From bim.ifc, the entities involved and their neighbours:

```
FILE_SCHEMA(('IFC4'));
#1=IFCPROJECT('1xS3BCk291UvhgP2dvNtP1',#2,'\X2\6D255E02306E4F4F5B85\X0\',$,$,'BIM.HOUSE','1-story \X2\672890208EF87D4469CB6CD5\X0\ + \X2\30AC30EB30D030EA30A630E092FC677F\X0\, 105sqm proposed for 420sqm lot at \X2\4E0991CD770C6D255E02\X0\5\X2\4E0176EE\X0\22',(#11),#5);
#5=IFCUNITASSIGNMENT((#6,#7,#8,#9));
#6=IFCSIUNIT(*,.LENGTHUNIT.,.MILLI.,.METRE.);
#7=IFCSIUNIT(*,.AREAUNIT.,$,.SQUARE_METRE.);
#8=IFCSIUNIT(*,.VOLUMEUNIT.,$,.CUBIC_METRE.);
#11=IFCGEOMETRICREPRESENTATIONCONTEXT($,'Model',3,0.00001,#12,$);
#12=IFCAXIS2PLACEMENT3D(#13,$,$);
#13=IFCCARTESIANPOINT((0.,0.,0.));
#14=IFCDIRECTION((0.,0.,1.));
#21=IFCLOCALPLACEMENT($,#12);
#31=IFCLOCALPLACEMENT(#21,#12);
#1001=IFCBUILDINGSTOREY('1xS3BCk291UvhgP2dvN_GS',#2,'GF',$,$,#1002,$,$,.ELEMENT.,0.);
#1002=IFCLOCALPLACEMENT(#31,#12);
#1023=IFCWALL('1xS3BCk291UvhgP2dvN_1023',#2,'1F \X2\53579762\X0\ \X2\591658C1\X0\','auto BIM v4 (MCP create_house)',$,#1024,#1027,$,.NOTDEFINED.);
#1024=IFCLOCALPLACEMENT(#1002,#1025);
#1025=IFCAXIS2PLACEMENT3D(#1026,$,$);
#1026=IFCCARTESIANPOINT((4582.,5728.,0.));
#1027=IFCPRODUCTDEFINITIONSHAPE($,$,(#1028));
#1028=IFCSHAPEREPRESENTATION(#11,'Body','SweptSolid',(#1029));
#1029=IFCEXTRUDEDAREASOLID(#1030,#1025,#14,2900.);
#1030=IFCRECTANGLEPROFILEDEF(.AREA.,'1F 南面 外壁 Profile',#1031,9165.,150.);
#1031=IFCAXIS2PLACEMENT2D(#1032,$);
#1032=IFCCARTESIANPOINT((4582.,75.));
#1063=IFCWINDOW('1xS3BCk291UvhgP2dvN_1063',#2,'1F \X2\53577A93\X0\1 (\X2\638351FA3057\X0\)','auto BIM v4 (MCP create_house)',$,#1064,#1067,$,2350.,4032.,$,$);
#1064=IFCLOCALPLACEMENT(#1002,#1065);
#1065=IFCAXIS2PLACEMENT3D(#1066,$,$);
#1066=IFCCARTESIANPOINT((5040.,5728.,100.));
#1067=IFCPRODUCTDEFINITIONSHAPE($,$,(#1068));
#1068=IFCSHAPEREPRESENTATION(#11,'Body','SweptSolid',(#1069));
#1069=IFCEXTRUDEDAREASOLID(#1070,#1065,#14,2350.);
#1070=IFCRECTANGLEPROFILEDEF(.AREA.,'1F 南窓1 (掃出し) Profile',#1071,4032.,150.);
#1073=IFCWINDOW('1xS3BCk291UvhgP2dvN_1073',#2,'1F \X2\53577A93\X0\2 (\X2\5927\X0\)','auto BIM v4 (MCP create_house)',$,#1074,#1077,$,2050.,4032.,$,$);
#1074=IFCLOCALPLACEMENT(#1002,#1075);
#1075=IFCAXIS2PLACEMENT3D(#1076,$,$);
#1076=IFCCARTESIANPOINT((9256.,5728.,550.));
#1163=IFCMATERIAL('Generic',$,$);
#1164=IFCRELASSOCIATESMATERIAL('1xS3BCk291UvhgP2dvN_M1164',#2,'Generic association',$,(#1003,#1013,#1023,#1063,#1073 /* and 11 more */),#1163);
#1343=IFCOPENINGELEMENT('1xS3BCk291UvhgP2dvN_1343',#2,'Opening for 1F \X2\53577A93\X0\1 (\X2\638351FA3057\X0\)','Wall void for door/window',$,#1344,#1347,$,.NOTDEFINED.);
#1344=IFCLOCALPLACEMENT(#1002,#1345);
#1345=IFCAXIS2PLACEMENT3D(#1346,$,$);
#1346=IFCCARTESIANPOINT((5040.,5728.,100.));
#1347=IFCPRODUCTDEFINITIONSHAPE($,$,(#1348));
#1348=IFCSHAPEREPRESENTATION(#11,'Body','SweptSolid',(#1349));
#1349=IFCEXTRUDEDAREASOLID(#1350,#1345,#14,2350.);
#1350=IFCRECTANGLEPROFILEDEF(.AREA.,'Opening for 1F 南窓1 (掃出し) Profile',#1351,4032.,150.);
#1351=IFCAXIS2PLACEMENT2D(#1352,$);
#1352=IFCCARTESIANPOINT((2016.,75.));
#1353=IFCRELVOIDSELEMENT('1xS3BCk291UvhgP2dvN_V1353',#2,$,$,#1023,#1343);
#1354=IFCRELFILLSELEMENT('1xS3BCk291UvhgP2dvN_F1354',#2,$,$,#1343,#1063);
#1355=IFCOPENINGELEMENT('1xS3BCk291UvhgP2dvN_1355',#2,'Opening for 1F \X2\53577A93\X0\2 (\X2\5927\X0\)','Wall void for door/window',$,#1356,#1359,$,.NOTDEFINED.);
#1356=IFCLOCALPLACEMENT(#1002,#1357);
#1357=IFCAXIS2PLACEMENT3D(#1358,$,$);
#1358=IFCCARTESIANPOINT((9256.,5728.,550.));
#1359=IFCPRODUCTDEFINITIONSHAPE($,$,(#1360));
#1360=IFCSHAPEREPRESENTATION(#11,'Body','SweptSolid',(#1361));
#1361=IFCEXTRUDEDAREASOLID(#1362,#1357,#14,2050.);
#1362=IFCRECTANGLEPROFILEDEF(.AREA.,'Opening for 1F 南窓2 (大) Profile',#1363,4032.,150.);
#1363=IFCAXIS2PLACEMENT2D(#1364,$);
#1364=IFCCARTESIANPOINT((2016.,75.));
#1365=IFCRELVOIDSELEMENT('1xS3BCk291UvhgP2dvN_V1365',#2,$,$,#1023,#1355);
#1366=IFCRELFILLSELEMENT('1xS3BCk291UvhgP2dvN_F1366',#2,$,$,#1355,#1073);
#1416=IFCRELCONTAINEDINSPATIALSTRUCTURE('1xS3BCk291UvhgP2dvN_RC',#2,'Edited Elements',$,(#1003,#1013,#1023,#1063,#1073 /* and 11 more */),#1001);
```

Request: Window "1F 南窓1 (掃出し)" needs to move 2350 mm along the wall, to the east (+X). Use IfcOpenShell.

```python
import ifcopenshell
import ifcopenshell.api.geometry
import ifcopenshell.util.placement
import ifcopenshell.util.unit

model = ifcopenshell.open("bim.ifc")
unit_scale = ifcopenshell.util.unit.calculate_unit_scale(model)

window = model.by_id(1063)
opening = window.FillsVoids[0].RelatingOpeningElement
wall = opening.VoidsElements[0].RelatingBuildingElement

wall_matrix = ifcopenshell.util.placement.get_local_placement(wall.ObjectPlacement)
shift = wall_matrix[:3, 0] * 2.35 / unit_scale
before = ifcopenshell.util.placement.get_local_placement(window.ObjectPlacement)[:3, 3].copy()

# The window is not placed relative to its opening, so move both.
for product in (opening, window):
    matrix = ifcopenshell.util.placement.get_local_placement(product.ObjectPlacement)
    matrix[:3, 3] += shift
    ifcopenshell.api.geometry.edit_object_placement(model, product=product, matrix=matrix, is_si=False)

after = ifcopenshell.util.placement.get_local_placement(window.ObjectPlacement)[:3, 3]
print("window moved by", (after - before).round(3) + 0.0)

model.write("bim-out.ifc")
```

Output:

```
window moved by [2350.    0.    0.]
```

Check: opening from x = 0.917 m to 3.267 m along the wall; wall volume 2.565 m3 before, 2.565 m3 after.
